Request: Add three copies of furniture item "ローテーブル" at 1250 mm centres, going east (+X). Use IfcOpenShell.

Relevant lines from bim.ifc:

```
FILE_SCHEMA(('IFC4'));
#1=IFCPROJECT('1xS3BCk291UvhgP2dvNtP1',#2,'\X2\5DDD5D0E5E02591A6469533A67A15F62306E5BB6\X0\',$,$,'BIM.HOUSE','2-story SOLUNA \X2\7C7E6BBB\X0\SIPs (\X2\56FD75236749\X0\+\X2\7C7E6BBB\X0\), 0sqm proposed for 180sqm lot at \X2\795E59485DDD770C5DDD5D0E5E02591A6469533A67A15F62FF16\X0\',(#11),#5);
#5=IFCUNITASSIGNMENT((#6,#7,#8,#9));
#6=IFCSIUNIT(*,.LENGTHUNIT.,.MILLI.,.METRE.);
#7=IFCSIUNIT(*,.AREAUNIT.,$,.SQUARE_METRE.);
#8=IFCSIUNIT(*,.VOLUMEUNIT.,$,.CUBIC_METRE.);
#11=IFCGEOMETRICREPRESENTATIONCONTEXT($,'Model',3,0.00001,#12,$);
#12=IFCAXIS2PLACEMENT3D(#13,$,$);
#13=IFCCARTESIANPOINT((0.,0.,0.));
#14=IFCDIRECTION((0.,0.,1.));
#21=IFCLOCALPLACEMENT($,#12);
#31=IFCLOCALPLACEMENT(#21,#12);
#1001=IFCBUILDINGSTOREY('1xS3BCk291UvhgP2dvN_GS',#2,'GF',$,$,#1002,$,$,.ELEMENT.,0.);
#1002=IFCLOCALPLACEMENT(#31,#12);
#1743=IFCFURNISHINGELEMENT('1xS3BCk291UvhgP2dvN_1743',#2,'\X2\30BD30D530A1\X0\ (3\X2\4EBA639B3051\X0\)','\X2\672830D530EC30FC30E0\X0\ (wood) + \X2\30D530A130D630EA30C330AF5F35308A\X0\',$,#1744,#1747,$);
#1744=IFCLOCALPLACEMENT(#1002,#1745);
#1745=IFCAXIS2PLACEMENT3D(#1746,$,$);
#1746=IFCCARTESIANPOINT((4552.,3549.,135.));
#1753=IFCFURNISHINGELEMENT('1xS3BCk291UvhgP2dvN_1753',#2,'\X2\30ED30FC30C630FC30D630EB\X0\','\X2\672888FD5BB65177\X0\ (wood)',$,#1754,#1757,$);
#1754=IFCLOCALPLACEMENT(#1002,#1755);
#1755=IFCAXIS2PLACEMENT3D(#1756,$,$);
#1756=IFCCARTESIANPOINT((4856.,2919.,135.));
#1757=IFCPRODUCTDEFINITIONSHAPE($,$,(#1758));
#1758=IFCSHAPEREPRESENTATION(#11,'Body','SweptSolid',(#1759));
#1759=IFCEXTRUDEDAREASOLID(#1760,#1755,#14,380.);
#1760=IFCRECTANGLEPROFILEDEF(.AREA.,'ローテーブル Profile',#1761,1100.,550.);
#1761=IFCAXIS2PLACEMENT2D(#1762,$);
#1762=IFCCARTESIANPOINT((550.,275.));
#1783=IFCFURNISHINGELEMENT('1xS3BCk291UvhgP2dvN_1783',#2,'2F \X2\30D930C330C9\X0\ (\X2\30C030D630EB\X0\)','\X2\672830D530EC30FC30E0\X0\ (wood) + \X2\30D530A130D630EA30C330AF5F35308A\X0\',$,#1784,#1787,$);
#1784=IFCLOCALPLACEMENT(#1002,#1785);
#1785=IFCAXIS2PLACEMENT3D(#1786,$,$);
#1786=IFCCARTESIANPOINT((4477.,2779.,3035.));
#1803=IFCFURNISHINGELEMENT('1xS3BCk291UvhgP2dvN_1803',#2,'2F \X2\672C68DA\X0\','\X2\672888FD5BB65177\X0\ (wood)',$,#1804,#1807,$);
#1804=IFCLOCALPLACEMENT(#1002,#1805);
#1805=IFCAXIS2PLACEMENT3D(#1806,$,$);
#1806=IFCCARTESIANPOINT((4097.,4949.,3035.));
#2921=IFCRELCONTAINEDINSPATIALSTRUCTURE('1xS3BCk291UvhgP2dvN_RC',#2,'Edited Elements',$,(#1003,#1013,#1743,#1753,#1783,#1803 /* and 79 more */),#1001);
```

```python
import numpy as np
import ifcopenshell
import ifcopenshell.api.geometry
import ifcopenshell.api.root
import ifcopenshell.util.element
import ifcopenshell.util.placement
import ifcopenshell.util.unit

model = ifcopenshell.open("bim.ifc")
unit_scale = ifcopenshell.util.unit.calculate_unit_scale(model)


def reuse_history(source, copy):
    """copy_class also copies each property set's owner history, people and application; keep the originals."""
    for rel in copy.IsDefinedBy:
        if rel.is_a("IfcRelDefinesByProperties") and (history := rel.RelatingPropertyDefinition.OwnerHistory):
            rel.RelatingPropertyDefinition.OwnerHistory = source.OwnerHistory
            ifcopenshell.util.element.remove_deep2(model, history)


source = model.by_id(1753)
base = ifcopenshell.util.placement.get_local_placement(source.ObjectPlacement)
step = np.array([1.0, 0.0, 0.0]) * 1.25 / unit_scale

for i in range(1, 4):
    copy = ifcopenshell.api.root.copy_class(model, product=source)
    copy.Representation = ifcopenshell.util.element.copy_deep(
        model, source.Representation, exclude=["IfcGeometricRepresentationContext", "IfcRepresentationMap"]
    )
    reuse_history(source, copy)
    matrix = base.copy()
    matrix[:3, 3] += i * step
    print("added at", matrix[:3, 3].round(3) + 0.0)
    ifcopenshell.api.geometry.edit_object_placement(model, product=copy, matrix=matrix, is_si=False)

model.write("bim_updated.ifc")
```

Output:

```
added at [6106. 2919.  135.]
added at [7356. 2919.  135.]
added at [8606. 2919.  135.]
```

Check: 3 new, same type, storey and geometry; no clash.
